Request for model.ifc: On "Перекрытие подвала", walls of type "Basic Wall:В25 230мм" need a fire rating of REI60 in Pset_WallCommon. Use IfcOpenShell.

First a look at what the model holds.

```python
import ifcopenshell
import ifcopenshell.util.element

model = ifcopenshell.open("model.ifc")
print(model.schema)
storey = next(s for s in model.by_type("IfcBuildingStorey") if s.Name == "Перекрытие подвала")
walls = [e for e in ifcopenshell.util.element.get_decomposition(storey) if e.is_a("IfcWall")]
seen = {}
for e in walls:
    element_type = ifcopenshell.util.element.get_type(e)
    key = (element_type.Name if element_type != e and element_type else None, ifcopenshell.util.element.get_pset(e, "Pset_WallCommon", "FireRating"))
    seen[key] = seen.get(key, 0) + 1
for (name, value), count in sorted(seen.items(), key=str):
    print(count, "x", name, "|", value)
```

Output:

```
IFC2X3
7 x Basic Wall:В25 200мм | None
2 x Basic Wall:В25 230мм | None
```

```python
import ifcopenshell
import ifcopenshell.api.pset
import ifcopenshell.util.element

model = ifcopenshell.open("model.ifc")

storey = next(s for s in model.by_type("IfcBuildingStorey") if s.Name == "Перекрытие подвала")
walls = [e for e in ifcopenshell.util.element.get_decomposition(storey) if e.is_a("IfcWall")]

count = 0
for e in walls:
    element_type = ifcopenshell.util.element.get_type(e)
    if element_type in (None, e) or element_type.Name != "Basic Wall:В25 230мм":
        continue
    # add_pset returns the element's existing set when there is one.
    pset = ifcopenshell.api.pset.add_pset(model, product=e, name="Pset_WallCommon")
    ifcopenshell.api.pset.edit_pset(model, pset=pset, properties={"FireRating": "REI60"})
    count += 1

print(count, "walls updated")

model.write("model_updated.ifc")
```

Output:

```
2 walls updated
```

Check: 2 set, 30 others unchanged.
